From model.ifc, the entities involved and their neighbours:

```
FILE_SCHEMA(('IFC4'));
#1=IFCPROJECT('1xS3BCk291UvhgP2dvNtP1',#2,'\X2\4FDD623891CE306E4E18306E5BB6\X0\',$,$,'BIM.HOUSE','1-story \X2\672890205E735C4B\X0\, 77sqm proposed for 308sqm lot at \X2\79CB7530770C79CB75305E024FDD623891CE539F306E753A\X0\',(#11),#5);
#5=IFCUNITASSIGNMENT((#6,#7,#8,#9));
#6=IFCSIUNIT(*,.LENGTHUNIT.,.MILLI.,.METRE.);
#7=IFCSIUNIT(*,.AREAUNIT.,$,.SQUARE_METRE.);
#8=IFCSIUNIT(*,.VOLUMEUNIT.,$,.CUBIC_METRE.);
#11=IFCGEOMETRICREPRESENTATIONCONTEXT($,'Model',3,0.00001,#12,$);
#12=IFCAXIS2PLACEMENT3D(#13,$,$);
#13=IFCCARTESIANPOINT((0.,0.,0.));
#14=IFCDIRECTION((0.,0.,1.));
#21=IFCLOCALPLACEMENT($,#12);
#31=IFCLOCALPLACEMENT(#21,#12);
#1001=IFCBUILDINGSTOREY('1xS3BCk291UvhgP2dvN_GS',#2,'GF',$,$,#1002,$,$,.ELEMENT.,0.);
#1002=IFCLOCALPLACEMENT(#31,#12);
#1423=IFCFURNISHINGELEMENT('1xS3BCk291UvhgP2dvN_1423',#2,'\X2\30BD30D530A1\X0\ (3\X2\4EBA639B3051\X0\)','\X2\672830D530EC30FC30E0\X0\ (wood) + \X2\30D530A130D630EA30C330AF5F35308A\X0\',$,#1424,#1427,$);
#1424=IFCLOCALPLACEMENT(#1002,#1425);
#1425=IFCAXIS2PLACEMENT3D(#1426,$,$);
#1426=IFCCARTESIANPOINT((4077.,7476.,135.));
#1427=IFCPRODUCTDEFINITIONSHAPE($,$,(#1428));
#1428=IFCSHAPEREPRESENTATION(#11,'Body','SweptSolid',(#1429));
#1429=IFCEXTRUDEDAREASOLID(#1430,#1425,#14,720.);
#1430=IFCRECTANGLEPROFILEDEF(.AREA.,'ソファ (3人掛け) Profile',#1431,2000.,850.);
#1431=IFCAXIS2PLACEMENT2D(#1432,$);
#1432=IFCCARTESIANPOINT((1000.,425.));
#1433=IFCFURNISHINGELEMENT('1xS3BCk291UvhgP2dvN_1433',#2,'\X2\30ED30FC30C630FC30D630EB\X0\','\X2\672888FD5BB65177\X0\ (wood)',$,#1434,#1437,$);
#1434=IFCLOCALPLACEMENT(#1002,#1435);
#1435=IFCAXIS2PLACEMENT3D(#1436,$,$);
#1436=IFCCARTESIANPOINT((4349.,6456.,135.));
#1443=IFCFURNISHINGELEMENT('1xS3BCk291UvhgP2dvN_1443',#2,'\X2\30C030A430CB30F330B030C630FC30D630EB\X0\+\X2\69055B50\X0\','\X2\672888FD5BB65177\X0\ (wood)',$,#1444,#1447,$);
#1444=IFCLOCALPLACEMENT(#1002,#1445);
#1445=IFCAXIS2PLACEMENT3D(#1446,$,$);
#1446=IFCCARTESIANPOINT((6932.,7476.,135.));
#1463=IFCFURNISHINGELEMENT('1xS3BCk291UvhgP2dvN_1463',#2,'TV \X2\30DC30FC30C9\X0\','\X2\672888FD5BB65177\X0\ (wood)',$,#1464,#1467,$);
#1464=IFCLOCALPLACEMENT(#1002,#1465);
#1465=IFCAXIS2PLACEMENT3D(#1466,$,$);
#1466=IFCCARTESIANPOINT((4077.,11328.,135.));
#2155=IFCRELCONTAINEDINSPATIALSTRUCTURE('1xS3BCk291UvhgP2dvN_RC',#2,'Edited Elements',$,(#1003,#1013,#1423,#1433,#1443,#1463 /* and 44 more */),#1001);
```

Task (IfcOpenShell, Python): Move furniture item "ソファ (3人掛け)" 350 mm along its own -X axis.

```python
import ifcopenshell
import ifcopenshell.api.geometry
import ifcopenshell.util.placement

model = ifcopenshell.open("model.ifc")

item = model.by_guid("1xS3BCk291UvhgP2dvN_1423")
matrix = ifcopenshell.util.placement.get_local_placement(item.ObjectPlacement)
matrix[:3, 3] -= matrix[:3, 0] * 350.0
ifcopenshell.api.geometry.edit_object_placement(model, product=item, matrix=matrix, is_si=False)

print(ifcopenshell.util.placement.get_local_placement(item.ObjectPlacement).round(3) + 0.0)

model.write("model-out.ifc")
```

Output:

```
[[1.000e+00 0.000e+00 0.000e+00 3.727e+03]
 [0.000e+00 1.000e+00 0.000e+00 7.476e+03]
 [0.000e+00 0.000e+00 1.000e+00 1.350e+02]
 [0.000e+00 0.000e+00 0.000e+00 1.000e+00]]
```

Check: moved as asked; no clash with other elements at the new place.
